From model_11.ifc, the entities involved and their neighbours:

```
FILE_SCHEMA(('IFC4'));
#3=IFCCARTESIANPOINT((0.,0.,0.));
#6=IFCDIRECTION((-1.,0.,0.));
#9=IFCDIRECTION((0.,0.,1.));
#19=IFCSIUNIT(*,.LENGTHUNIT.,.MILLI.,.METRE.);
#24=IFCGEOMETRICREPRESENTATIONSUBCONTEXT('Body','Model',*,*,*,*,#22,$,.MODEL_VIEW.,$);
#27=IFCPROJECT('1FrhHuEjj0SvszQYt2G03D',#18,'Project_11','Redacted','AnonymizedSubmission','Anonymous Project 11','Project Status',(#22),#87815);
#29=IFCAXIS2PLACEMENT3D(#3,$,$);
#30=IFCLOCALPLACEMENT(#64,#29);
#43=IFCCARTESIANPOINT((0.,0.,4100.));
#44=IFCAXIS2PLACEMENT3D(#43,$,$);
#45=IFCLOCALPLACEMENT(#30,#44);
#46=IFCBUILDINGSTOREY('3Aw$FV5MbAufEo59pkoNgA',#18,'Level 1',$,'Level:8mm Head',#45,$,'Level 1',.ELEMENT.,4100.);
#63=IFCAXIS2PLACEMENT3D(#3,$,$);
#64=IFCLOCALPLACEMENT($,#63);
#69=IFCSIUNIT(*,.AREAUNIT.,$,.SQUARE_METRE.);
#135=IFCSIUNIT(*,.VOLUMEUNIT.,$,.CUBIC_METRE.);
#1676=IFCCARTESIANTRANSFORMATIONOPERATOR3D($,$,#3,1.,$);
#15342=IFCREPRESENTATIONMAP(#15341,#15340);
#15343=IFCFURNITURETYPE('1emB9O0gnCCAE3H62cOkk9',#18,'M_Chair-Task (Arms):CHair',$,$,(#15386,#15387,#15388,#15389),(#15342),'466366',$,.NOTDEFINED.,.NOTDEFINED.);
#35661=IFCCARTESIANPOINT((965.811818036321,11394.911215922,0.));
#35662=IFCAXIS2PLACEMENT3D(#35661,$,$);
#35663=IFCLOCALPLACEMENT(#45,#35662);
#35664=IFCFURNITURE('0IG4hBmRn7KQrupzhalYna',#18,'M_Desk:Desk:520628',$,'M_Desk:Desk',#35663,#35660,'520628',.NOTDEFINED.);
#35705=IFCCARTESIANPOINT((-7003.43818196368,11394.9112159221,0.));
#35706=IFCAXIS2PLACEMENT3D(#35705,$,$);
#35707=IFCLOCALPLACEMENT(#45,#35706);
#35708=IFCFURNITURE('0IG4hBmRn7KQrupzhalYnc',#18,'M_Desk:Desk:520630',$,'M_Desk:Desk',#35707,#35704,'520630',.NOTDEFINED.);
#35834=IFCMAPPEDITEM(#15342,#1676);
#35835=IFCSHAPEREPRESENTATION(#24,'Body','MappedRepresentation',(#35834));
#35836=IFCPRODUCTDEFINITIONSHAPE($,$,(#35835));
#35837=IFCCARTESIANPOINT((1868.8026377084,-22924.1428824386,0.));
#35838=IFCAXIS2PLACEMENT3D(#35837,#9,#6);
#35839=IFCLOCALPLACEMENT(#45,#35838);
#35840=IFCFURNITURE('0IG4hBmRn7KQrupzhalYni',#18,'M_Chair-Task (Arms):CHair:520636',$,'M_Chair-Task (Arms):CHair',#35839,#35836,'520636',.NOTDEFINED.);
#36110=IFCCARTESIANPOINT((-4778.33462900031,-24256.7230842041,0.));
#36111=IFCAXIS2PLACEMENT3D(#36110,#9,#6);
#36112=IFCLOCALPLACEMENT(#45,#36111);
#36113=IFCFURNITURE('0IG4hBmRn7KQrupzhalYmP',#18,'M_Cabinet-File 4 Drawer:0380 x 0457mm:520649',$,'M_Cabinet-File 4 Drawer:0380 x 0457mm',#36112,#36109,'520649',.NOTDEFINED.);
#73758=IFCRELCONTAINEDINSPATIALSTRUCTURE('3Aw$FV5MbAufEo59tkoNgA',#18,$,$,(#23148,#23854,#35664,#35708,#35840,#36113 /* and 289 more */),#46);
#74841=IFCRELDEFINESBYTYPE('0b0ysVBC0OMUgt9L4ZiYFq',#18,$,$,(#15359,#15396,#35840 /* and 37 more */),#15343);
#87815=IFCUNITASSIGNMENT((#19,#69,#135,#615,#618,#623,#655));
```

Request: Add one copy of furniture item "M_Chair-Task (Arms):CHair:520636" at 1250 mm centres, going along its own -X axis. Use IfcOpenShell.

```python
import ifcopenshell
import ifcopenshell.api.geometry
import ifcopenshell.api.root
import ifcopenshell.util.element
import ifcopenshell.util.placement

model = ifcopenshell.open("model_11.ifc")


def reuse_history(source, copy):
    """copy_class also copies each property set's owner history, people and application; keep the originals."""
    for rel in copy.IsDefinedBy:
        if rel.is_a("IfcRelDefinesByProperties") and (history := rel.RelatingPropertyDefinition.OwnerHistory):
            rel.RelatingPropertyDefinition.OwnerHistory = source.OwnerHistory
            ifcopenshell.util.element.remove_deep2(model, history)


source = model.by_guid("0IG4hBmRn7KQrupzhalYni")
base = ifcopenshell.util.placement.get_local_placement(source.ObjectPlacement)
step = -base[:3, 0] * 1250.0

for i in range(1, 2):
    copy = ifcopenshell.api.root.copy_class(model, product=source)
    copy.Representation = ifcopenshell.util.element.copy_deep(
        model, source.Representation, exclude=["IfcGeometricRepresentationContext", "IfcRepresentationMap"]
    )
    copy.Name = "M_Chair-Task (Arms):CHair"
    copy.Tag = None
    reuse_history(source, copy)
    matrix = base.copy()
    matrix[:3, 3] += i * step
    print("added at", matrix[:3, 3].round(3) + 0.0)
    ifcopenshell.api.geometry.edit_object_placement(model, product=copy, matrix=matrix, is_si=False)

model.write("model_11_rev.ifc")
```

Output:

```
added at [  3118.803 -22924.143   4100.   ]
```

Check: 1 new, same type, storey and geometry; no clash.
